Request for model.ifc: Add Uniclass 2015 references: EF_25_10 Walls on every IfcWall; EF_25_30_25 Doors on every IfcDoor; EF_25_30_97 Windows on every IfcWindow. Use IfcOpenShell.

First a look at what the model holds.

```python
import ifcopenshell

model = ifcopenshell.open("model.ifc")
print(model.schema)
print("classifications:", [c.Name for c in model.by_type("IfcClassification")])
for ifc_class in ("IfcDoor", "IfcRoof", "IfcStair", "IfcWall", "IfcWindow"):
    print(ifc_class, len(model.by_type(ifc_class)))
```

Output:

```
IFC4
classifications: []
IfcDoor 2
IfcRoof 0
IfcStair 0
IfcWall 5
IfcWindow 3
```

```python
import ifcopenshell
import ifcopenshell.api.classification

model = ifcopenshell.open("model.ifc")

system = ifcopenshell.api.classification.add_classification(model, classification="Uniclass 2015")

codes = {
    "IfcWall": ("EF_25_10", "Walls"),
    "IfcDoor": ("EF_25_30_25", "Doors"),
    "IfcWindow": ("EF_25_30_97", "Windows"),
}
for ifc_class, (code, name) in codes.items():
    products = model.by_type(ifc_class)
    ifcopenshell.api.classification.add_reference(
        model, products=products, classification=system, identification=code, name=name
    )
    print(code, len(products))

model.write("model_updated.ifc")
```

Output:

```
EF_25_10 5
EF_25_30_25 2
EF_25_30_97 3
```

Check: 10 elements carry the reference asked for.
